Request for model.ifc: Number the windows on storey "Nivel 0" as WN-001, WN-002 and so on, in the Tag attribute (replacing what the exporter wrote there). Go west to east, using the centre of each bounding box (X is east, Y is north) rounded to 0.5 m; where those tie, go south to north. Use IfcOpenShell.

First a look at what the model holds.

```python
import ifcopenshell
import ifcopenshell.util.element
import ifcopenshell.util.placement

model = ifcopenshell.open("model.ifc")
print(model.schema)
storey = next(s for s in model.by_type("IfcBuildingStorey") if s.Name == "Nivel 0")
windows = [e for e in ifcopenshell.util.element.get_decomposition(storey) if e.is_a("IfcWindow")]
for e in sorted(windows, key=lambda e: e.id()):
    origin = ifcopenshell.util.placement.get_local_placement(e.ObjectPlacement)[:3, 3]
    print(e.id(), e.Tag, e.Name, origin.round(2) + 0.0, sep=" | ")
```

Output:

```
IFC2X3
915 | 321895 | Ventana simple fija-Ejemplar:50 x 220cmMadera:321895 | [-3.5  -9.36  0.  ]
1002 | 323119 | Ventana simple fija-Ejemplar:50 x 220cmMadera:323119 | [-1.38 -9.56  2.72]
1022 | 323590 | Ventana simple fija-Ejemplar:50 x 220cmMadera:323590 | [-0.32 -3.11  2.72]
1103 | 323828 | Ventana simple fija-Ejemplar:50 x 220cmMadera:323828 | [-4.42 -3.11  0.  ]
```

```python
import ifcopenshell
import ifcopenshell.geom
import ifcopenshell.util.element
import ifcopenshell.util.shape

model = ifcopenshell.open("model.ifc")
settings = ifcopenshell.geom.settings()
settings.set("use-world-coords", True)


def centre(element):
    shape = ifcopenshell.geom.create_shape(settings, element)
    return ifcopenshell.util.shape.get_bbox_centroid(shape.geometry)


storey = next(s for s in model.by_type("IfcBuildingStorey") if s.Name == "Nivel 0")
windows = [e for e in ifcopenshell.util.element.get_decomposition(storey) if e.is_a("IfcWindow")]

# Insertion points can sit at a corner or the storey origin, so sort by the geometry (in metres).
centres = {e: centre(e) for e in windows}
windows.sort(key=lambda e: (round(centres[e][0] / 0.5), centres[e][1]))

for i, e in enumerate(windows, start=1):
    number = f"WN-0{i:02d}"
    e.Tag = number
    print(e.id(), number)

model.write("model_updated.ifc")
```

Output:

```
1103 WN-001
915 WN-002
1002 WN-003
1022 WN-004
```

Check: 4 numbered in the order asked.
